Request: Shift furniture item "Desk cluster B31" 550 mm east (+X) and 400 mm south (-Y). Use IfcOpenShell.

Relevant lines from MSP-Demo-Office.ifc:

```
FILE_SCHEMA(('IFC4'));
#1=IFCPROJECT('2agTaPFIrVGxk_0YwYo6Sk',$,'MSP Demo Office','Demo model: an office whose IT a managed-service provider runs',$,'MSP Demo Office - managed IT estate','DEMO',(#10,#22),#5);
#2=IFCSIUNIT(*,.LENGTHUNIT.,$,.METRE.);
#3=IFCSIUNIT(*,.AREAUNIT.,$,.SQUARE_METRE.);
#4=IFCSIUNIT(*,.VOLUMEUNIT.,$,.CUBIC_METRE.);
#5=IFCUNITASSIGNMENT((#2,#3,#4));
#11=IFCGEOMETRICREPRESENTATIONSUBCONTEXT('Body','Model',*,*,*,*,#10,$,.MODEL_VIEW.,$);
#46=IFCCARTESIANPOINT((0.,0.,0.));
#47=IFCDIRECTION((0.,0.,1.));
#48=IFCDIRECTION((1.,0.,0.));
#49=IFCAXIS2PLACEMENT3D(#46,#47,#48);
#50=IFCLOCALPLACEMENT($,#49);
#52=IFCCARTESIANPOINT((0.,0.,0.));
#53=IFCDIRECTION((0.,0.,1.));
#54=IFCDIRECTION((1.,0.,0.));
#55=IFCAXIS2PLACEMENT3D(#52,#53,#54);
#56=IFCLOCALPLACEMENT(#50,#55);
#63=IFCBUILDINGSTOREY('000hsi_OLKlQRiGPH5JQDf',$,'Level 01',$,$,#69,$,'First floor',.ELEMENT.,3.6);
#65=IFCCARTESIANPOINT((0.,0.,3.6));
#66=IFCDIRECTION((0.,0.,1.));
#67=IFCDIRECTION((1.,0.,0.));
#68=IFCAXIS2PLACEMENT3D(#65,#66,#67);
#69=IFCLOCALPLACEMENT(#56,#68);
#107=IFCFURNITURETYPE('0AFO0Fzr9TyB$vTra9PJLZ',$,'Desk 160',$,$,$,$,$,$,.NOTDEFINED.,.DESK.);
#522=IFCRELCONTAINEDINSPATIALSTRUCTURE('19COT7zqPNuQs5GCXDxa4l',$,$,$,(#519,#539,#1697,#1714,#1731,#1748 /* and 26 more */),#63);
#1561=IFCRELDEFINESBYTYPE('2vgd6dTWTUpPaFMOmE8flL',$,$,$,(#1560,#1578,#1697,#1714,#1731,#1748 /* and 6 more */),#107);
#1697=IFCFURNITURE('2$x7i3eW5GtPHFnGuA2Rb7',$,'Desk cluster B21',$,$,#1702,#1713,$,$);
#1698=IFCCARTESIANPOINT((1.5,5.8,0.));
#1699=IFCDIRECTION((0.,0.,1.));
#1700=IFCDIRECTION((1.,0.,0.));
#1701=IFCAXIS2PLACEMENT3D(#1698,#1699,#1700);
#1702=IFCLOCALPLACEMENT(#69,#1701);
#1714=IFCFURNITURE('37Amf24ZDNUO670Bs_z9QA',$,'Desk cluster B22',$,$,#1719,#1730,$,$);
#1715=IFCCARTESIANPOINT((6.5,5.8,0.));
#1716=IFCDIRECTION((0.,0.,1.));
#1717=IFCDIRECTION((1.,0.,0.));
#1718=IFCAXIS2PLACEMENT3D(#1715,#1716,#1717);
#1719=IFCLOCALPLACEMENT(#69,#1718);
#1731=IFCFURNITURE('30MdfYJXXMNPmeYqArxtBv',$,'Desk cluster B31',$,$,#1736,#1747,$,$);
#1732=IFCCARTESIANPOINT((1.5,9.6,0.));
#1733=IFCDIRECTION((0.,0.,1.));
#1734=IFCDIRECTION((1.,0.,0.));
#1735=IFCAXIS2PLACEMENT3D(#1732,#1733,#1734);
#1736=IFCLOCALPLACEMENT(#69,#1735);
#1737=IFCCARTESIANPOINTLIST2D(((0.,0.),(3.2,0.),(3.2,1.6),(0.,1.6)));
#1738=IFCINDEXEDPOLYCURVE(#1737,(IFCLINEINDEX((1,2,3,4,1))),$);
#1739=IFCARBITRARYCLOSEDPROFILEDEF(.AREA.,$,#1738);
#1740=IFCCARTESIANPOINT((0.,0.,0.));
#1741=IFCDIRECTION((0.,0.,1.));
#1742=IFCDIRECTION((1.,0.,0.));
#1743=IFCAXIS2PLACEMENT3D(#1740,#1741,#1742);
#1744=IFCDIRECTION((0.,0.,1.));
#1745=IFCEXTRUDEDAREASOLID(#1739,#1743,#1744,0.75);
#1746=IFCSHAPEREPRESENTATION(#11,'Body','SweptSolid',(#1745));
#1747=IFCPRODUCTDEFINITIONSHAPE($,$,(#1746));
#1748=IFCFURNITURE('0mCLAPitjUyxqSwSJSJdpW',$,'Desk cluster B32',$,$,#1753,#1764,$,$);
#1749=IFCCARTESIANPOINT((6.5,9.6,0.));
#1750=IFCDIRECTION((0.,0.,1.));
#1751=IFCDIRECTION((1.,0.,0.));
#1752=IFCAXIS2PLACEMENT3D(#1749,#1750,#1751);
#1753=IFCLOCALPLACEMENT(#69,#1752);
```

```python
import ifcopenshell
import ifcopenshell.api.geometry
import ifcopenshell.util.placement

model = ifcopenshell.open("MSP-Demo-Office.ifc")

item = model.by_guid("30MdfYJXXMNPmeYqArxtBv")
matrix = ifcopenshell.util.placement.get_local_placement(item.ObjectPlacement)
matrix[0, 3] += 0.55
matrix[1, 3] -= 0.4
ifcopenshell.api.geometry.edit_object_placement(model, product=item, matrix=matrix, is_si=False)

print(ifcopenshell.util.placement.get_local_placement(item.ObjectPlacement).round(3) + 0.0)

model.write("MSP-Demo-Office_edited.ifc")
```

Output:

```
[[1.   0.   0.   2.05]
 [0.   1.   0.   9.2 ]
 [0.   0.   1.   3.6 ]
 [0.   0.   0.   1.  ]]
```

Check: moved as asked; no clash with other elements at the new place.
